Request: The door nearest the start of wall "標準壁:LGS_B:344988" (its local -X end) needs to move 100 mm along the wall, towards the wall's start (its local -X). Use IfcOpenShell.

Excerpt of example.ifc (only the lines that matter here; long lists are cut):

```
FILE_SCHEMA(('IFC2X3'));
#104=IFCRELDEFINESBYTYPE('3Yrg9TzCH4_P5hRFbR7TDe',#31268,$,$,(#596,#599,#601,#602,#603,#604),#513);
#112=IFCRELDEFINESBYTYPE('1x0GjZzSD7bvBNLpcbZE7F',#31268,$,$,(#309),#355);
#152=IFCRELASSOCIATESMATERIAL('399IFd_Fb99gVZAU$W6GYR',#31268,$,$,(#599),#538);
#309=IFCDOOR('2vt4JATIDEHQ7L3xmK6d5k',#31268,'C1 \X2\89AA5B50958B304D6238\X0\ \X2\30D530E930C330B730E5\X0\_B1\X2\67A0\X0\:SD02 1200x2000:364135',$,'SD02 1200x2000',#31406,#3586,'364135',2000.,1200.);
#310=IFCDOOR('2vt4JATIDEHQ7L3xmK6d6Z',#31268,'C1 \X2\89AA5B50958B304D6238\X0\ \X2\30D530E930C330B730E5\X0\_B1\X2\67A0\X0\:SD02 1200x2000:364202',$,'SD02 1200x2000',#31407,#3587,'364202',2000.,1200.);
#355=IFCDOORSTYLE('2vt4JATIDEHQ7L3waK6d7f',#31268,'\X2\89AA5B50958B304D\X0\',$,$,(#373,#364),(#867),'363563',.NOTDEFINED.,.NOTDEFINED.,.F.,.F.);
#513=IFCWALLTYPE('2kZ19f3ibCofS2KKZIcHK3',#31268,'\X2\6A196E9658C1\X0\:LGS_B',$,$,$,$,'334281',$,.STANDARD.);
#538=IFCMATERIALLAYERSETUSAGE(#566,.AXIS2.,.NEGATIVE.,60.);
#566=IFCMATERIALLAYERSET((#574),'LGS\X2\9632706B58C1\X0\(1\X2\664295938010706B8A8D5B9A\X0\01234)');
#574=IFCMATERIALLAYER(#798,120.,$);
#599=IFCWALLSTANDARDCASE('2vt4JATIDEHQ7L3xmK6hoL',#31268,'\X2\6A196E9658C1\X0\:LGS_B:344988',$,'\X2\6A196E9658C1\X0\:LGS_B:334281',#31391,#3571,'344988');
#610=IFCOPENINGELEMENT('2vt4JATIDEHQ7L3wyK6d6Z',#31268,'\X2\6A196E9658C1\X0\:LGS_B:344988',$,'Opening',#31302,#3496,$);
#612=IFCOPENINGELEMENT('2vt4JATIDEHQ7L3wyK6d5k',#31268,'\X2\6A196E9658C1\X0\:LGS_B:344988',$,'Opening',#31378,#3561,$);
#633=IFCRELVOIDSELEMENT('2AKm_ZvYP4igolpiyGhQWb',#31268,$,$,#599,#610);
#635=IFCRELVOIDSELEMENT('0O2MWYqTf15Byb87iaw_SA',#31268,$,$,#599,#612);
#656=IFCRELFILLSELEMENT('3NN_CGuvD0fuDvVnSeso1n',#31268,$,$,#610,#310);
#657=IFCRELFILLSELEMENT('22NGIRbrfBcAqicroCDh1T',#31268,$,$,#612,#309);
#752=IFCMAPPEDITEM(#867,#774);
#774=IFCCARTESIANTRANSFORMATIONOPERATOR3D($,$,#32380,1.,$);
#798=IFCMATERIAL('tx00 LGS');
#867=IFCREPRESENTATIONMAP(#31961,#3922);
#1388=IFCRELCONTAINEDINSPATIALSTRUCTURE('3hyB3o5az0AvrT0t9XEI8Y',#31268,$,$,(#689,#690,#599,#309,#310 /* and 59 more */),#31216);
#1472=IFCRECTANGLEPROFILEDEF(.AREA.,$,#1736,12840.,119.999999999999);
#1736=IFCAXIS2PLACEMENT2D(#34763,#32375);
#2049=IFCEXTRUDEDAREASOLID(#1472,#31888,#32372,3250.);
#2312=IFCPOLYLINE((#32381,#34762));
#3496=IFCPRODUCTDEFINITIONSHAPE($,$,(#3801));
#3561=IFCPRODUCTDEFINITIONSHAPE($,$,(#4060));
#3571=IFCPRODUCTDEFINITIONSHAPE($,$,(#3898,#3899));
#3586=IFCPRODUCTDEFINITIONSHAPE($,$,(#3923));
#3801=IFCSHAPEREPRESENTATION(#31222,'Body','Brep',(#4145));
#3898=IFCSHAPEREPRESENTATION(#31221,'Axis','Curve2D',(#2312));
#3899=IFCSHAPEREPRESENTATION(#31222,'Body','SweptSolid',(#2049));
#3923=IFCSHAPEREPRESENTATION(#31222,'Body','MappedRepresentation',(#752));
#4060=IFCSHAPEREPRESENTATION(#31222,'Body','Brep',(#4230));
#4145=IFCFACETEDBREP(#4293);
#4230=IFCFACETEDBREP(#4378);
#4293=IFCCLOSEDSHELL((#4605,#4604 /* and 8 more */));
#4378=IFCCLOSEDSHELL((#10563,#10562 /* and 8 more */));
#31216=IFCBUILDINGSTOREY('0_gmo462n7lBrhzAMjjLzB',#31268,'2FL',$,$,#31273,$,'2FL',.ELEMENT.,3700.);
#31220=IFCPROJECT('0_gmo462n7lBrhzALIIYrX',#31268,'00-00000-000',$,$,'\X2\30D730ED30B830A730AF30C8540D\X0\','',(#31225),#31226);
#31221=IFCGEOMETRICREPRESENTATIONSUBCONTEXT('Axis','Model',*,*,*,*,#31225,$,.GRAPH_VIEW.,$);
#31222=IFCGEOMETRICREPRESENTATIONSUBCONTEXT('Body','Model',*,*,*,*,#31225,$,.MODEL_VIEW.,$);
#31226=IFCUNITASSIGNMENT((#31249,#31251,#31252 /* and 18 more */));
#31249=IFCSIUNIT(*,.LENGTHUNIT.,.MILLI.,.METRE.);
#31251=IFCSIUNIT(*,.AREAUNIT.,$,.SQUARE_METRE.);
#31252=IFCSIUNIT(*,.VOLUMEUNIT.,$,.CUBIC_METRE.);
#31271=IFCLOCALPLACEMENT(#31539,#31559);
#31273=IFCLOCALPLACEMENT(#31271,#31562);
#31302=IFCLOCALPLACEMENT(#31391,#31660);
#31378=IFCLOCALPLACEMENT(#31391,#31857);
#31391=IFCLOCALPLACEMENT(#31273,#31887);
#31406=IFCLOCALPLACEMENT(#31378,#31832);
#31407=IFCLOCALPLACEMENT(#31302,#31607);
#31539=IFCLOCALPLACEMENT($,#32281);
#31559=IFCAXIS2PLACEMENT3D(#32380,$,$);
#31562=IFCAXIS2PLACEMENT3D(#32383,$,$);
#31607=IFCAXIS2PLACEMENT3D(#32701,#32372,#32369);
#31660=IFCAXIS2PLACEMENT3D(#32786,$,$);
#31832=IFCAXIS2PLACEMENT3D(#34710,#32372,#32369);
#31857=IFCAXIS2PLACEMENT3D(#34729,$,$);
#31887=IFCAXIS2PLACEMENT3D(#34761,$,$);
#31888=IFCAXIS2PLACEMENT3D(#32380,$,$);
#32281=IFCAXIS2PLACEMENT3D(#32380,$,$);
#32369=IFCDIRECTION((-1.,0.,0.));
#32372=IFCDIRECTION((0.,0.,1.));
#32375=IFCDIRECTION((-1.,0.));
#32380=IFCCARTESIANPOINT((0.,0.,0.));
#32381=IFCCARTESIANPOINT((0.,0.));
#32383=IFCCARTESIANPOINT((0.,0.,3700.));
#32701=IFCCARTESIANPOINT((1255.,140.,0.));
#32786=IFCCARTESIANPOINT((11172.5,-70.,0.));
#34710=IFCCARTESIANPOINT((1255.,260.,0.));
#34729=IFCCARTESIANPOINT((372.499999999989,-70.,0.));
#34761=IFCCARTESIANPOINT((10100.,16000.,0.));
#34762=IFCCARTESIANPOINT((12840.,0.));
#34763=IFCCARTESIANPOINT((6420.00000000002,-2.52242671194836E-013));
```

```python
import ifcopenshell
import ifcopenshell.api.geometry
import ifcopenshell.util.placement
import ifcopenshell.util.unit

model = ifcopenshell.open("example.ifc")
unit_scale = ifcopenshell.util.unit.calculate_unit_scale(model)

door = model.by_guid("2vt4JATIDEHQ7L3xmK6d5k")
opening = door.FillsVoids[0].RelatingOpeningElement
wall = opening.VoidsElements[0].RelatingBuildingElement

wall_matrix = ifcopenshell.util.placement.get_local_placement(wall.ObjectPlacement)
shift = wall_matrix[:3, 0] * -0.1 / unit_scale
before = ifcopenshell.util.placement.get_local_placement(door.ObjectPlacement)[:3, 3].copy()

# The door is placed relative to its opening, so it follows when the opening moves.
matrix = ifcopenshell.util.placement.get_local_placement(opening.ObjectPlacement)
matrix[:3, 3] += shift
ifcopenshell.api.geometry.edit_object_placement(
    model, product=opening, matrix=matrix, is_si=False, should_transform_children=True
)

after = ifcopenshell.util.placement.get_local_placement(door.ObjectPlacement)[:3, 3]
print("door moved by", (after - before).round(3) + 0.0)

model.write("example-out.ifc")
```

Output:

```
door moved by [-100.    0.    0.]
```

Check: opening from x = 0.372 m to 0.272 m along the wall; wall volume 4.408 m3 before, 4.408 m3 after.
